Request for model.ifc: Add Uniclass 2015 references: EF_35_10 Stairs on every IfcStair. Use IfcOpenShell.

First a look at what the model holds.

```python
import ifcopenshell

model = ifcopenshell.open("model.ifc")
print(model.schema)
print("classifications:", [c.Name for c in model.by_type("IfcClassification")])
for ifc_class in ("IfcDoor", "IfcRoof", "IfcStair", "IfcWall", "IfcWindow"):
    print(ifc_class, len(model.by_type(ifc_class)))
```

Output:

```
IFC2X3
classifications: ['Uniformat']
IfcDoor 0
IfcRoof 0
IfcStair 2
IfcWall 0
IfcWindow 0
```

```python
import ifcopenshell
import ifcopenshell.api.classification

model = ifcopenshell.open("model.ifc")

# IFC2X3 requires Source and Edition and has no link from the project to the system.
system = model.create_entity("IfcClassification", Source="NBS", Edition="2015", Name="Uniclass 2015")

codes = {
    "IfcStair": ("EF_35_10", "Stairs"),
}
for ifc_class, (code, name) in codes.items():
    products = model.by_type(ifc_class)
    ifcopenshell.api.classification.add_reference(
        model, products=products, classification=system, identification=code, name=name
    )
    print(code, len(products))

model.write("model-out.ifc")
```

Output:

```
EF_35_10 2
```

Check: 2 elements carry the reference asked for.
